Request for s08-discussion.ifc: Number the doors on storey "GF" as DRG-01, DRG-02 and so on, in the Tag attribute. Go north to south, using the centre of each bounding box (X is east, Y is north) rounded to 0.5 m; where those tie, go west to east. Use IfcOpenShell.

First a look at what the model holds.

```python
import ifcopenshell
import ifcopenshell.util.element
import ifcopenshell.util.placement

model = ifcopenshell.open("s08-discussion.ifc")
print(model.schema)
storey = next(s for s in model.by_type("IfcBuildingStorey") if s.Name == "GF")
doors = [e for e in ifcopenshell.util.element.get_decomposition(storey) if e.is_a("IfcDoor")]
for e in sorted(doors, key=lambda e: e.id()):
    origin = ifcopenshell.util.placement.get_local_placement(e.ObjectPlacement)[:3, 3]
    print(e.id(), e.Tag, e.Name, origin.round(2) + 0.0, sep=" | ")
```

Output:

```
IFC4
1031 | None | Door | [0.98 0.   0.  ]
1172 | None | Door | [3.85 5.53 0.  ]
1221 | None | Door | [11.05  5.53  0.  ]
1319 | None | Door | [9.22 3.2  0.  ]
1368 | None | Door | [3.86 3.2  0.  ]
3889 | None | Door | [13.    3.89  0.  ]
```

```python
import ifcopenshell
import ifcopenshell.geom
import ifcopenshell.util.element
import ifcopenshell.util.shape

model = ifcopenshell.open("s08-discussion.ifc")
settings = ifcopenshell.geom.settings()
settings.set("use-world-coords", True)


def centre(element):
    shape = ifcopenshell.geom.create_shape(settings, element)
    return ifcopenshell.util.shape.get_bbox_centroid(shape.geometry)


storey = next(s for s in model.by_type("IfcBuildingStorey") if s.Name == "GF")
doors = [e for e in ifcopenshell.util.element.get_decomposition(storey) if e.is_a("IfcDoor")]

# Insertion points can sit at a corner or the storey origin, so sort by the geometry (in metres).
centres = {e: centre(e) for e in doors}
doors.sort(key=lambda e: (-round(centres[e][1] / 0.5), centres[e][0]))

for i, e in enumerate(doors, start=1):
    number = f"DRG-{i:02d}"
    e.Tag = number
    print(e.id(), number)

model.write("s08-discussion_v2.ifc")
```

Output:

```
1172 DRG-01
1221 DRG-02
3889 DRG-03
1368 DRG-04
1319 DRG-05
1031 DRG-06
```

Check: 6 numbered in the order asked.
